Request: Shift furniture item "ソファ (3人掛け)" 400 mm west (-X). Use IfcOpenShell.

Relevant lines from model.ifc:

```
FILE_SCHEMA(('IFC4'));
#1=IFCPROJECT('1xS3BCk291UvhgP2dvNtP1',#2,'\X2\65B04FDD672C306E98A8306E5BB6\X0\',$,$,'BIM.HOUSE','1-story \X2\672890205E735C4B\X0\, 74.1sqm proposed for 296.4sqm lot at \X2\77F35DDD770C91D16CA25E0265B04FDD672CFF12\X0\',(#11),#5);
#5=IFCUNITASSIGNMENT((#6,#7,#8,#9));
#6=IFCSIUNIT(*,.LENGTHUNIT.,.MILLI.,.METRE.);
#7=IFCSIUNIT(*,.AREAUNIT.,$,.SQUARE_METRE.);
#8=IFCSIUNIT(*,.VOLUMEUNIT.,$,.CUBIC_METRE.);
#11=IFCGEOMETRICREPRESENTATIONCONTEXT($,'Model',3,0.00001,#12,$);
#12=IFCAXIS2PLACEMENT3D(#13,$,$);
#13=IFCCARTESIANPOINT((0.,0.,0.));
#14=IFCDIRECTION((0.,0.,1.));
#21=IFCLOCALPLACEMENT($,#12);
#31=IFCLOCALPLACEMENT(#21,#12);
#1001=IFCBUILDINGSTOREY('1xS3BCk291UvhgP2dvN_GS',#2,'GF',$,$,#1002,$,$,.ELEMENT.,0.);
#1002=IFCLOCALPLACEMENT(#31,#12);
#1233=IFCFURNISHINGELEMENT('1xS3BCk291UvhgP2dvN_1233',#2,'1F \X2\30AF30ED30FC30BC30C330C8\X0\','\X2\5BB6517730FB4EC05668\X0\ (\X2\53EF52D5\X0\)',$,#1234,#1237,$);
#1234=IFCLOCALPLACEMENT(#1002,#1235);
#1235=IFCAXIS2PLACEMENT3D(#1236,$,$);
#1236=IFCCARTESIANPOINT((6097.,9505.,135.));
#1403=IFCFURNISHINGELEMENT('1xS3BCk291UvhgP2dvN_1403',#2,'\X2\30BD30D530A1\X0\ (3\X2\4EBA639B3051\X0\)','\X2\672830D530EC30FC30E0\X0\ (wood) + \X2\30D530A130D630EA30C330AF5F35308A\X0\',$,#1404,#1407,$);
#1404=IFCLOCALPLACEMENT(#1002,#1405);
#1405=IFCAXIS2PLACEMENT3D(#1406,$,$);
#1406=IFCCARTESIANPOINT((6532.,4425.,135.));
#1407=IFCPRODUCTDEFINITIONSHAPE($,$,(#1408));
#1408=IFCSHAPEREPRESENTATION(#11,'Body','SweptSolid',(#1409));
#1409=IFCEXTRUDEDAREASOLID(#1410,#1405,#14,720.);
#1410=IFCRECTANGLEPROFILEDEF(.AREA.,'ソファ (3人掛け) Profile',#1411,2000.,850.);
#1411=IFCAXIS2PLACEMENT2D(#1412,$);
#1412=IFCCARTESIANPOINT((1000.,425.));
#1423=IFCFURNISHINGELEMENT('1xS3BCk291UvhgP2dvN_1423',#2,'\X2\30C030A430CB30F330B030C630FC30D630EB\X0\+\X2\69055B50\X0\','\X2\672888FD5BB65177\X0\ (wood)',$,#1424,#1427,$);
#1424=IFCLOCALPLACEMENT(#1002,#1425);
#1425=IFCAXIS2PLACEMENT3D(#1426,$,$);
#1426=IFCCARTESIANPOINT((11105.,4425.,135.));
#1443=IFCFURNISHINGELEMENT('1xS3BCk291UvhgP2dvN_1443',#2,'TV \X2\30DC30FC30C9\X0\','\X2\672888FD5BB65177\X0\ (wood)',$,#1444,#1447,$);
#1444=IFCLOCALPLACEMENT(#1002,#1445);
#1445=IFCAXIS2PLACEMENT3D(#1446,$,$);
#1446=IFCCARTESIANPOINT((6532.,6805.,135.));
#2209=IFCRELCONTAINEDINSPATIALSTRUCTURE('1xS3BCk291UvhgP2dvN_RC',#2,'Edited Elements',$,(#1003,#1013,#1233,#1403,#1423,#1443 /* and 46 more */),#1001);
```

```python
import ifcopenshell
import ifcopenshell.api.geometry
import ifcopenshell.util.placement

model = ifcopenshell.open("model.ifc")

item = model.by_guid("1xS3BCk291UvhgP2dvN_1403")
matrix = ifcopenshell.util.placement.get_local_placement(item.ObjectPlacement)
matrix[0, 3] -= 400.0
ifcopenshell.api.geometry.edit_object_placement(model, product=item, matrix=matrix, is_si=False)

print(ifcopenshell.util.placement.get_local_placement(item.ObjectPlacement).round(3) + 0.0)

model.write("model-out.ifc")
```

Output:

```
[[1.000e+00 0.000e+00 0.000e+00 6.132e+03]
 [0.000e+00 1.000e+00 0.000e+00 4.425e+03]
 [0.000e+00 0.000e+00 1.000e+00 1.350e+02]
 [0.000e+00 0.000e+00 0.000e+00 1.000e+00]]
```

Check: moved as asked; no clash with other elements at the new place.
